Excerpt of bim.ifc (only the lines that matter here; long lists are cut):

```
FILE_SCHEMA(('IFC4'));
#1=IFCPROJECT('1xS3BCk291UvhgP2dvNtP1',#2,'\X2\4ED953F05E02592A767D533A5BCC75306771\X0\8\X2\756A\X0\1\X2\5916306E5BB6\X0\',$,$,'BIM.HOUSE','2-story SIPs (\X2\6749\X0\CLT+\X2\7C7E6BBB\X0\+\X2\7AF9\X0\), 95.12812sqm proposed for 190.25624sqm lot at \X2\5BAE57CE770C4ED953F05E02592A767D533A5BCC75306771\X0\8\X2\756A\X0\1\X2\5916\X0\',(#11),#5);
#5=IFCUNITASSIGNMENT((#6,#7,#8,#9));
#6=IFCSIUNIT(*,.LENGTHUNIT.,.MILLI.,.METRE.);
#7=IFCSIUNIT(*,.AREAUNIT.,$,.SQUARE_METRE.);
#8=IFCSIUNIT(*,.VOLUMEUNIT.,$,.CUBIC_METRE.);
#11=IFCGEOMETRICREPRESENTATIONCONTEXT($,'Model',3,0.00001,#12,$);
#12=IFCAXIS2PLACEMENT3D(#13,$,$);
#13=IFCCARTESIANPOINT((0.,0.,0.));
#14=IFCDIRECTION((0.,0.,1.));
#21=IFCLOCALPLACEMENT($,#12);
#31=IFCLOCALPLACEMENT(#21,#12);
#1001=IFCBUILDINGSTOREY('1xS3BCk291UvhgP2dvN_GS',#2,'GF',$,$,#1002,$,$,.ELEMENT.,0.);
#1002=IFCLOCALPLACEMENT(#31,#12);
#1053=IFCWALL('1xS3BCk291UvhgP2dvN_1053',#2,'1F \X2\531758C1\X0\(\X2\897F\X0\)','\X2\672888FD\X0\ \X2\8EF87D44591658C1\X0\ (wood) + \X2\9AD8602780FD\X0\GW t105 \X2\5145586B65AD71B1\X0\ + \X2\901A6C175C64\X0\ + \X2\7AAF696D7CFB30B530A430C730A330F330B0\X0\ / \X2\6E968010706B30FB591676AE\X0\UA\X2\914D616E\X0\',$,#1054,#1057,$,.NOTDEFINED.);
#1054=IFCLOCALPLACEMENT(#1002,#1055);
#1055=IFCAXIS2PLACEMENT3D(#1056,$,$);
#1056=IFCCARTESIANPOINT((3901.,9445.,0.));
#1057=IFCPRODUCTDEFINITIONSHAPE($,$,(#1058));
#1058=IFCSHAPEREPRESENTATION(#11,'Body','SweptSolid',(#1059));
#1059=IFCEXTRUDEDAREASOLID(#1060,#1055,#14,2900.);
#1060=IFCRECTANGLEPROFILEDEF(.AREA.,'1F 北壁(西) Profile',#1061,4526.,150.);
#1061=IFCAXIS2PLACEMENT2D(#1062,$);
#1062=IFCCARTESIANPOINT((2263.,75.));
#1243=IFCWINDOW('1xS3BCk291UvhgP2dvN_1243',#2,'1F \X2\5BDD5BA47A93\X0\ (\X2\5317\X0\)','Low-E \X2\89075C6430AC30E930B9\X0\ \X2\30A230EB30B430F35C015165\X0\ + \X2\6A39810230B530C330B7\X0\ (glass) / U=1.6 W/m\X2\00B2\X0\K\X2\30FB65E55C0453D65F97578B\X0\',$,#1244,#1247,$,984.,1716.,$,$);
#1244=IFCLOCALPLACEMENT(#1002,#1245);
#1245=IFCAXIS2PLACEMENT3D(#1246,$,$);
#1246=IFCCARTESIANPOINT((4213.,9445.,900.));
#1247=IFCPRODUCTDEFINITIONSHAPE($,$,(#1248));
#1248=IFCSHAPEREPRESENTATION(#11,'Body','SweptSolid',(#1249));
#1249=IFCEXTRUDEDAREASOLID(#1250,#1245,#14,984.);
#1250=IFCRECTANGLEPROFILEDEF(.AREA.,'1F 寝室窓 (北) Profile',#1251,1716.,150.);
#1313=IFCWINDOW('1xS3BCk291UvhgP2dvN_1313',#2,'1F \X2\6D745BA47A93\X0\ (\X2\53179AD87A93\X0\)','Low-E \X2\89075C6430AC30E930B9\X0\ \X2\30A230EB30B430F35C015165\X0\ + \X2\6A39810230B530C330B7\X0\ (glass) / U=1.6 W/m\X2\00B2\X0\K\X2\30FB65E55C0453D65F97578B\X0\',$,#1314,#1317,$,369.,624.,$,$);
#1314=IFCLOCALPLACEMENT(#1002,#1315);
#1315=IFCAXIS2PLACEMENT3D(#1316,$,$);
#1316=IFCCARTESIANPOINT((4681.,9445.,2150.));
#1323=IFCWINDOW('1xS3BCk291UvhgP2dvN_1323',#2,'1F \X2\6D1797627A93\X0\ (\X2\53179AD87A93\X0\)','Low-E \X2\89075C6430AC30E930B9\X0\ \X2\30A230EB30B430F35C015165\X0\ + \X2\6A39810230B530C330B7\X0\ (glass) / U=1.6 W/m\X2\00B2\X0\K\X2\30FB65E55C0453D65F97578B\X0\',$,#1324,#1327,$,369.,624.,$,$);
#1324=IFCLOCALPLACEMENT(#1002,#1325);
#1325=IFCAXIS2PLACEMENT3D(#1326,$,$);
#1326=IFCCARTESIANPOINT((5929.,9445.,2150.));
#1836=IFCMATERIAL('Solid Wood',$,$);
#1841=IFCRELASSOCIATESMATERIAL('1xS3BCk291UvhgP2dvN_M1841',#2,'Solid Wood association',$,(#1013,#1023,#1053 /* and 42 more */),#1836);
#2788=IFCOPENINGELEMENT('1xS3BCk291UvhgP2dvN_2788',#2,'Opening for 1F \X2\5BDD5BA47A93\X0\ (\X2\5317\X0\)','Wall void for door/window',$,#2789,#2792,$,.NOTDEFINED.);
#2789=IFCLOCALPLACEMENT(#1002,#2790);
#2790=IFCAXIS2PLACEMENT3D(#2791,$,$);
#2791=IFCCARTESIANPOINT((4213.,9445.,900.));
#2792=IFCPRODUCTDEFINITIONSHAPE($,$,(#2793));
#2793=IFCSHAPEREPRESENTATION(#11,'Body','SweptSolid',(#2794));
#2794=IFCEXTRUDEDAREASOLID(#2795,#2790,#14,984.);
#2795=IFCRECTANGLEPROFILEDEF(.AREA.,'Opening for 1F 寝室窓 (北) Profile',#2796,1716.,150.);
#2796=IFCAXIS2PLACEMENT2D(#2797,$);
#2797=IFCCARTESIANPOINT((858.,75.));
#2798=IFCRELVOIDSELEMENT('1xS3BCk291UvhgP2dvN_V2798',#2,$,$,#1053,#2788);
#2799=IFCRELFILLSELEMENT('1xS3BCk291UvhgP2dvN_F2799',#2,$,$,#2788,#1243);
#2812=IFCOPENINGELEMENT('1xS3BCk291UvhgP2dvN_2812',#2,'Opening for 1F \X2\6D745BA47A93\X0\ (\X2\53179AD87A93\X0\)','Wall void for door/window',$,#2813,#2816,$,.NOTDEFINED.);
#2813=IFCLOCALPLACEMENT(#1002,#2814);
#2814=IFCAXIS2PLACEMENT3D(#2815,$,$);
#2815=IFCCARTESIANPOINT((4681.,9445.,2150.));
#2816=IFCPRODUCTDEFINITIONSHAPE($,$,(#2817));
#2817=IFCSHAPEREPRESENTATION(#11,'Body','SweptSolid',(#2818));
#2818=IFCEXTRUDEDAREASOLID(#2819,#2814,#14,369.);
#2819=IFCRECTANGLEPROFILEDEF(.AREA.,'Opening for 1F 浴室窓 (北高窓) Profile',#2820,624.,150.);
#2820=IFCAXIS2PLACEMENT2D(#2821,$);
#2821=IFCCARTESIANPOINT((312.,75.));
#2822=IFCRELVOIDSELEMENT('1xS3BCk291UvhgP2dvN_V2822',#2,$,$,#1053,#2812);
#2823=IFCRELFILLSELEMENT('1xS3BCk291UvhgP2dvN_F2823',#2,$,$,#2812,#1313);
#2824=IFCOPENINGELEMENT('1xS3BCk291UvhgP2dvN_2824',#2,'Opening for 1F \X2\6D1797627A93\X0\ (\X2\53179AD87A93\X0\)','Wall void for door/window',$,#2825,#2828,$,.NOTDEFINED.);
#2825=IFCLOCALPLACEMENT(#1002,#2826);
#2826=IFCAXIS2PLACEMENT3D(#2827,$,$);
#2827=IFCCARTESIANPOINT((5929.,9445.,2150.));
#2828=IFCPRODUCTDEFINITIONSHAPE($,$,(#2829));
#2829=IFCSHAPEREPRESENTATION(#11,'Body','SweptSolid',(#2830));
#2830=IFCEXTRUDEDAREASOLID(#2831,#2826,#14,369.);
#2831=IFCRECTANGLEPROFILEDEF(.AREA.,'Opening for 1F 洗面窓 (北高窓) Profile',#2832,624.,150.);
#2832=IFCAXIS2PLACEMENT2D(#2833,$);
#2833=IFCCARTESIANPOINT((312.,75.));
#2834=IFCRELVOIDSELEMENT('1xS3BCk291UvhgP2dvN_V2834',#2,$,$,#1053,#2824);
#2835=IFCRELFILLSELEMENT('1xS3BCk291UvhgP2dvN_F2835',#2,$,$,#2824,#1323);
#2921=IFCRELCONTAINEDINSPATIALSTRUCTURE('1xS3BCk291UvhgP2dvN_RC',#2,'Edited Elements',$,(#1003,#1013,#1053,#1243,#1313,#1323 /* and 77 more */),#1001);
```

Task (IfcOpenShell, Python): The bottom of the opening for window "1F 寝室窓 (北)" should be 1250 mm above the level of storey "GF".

```python
import numpy as np
import ifcopenshell
import ifcopenshell.api.geometry
import ifcopenshell.geom
import ifcopenshell.util.element
import ifcopenshell.util.placement
import ifcopenshell.util.shape
import ifcopenshell.util.unit

model = ifcopenshell.open("bim.ifc")
unit_scale = ifcopenshell.util.unit.calculate_unit_scale(model)

window = model.by_id(1243)
opening = window.FillsVoids[0].RelatingOpeningElement
storey = ifcopenshell.util.element.get_container(window, ifc_class="IfcBuildingStorey")
level = ifcopenshell.util.placement.get_local_placement(storey.ObjectPlacement)[2, 3]

# The opening's origin need not be at the sill, so measure its lowest point.
shape = ifcopenshell.geom.create_shape(ifcopenshell.geom.settings(), opening)
bottom = ifcopenshell.util.shape.get_shape_bottom_elevation(shape, shape.geometry) / unit_scale
dz = level + 1.25 / unit_scale - bottom

shift = np.array([0.0, 0.0, dz])
# The window is not placed relative to its opening, so move both.
for product in (opening, window):
    matrix = ifcopenshell.util.placement.get_local_placement(product.ObjectPlacement)
    matrix[:3, 3] += shift
    ifcopenshell.api.geometry.edit_object_placement(model, product=product, matrix=matrix, is_si=False)

print(f"moved by {dz * unit_scale:+.3f} m")

model.write("bim_edited.ifc")
```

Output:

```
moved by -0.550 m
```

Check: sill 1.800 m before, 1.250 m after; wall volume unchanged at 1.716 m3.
